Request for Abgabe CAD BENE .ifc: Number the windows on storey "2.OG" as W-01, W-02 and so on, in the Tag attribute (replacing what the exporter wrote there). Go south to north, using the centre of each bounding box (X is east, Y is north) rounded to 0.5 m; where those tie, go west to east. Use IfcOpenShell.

First a look at what the model holds.

```python
import ifcopenshell
import ifcopenshell.util.element
import ifcopenshell.util.placement

model = ifcopenshell.open("Abgabe CAD BENE .ifc")
print(model.schema)
storey = next(s for s in model.by_type("IfcBuildingStorey") if s.Name == "2.OG")
windows = [e for e in ifcopenshell.util.element.get_decomposition(storey) if e.is_a("IfcWindow")]
for e in sorted(windows, key=lambda e: e.id()):
    origin = ifcopenshell.util.placement.get_local_placement(e.ObjectPlacement)[:3, 3]
    print(e.id(), e.Tag, e.Name, origin.round(2) + 0.0, sep=" | ")
```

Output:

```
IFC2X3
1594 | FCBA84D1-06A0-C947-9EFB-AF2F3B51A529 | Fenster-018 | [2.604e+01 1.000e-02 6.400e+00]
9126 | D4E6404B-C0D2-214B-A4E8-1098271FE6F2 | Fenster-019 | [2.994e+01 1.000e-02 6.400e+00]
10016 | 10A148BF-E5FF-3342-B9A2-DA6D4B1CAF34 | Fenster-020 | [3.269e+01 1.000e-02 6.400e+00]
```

```python
import ifcopenshell
import ifcopenshell.geom
import ifcopenshell.util.element
import ifcopenshell.util.shape

model = ifcopenshell.open("Abgabe CAD BENE .ifc")
settings = ifcopenshell.geom.settings()
settings.set("use-world-coords", True)


def centre(element):
    shape = ifcopenshell.geom.create_shape(settings, element)
    return ifcopenshell.util.shape.get_bbox_centroid(shape.geometry)


storey = next(s for s in model.by_type("IfcBuildingStorey") if s.Name == "2.OG")
windows = [e for e in ifcopenshell.util.element.get_decomposition(storey) if e.is_a("IfcWindow")]

# Insertion points can sit at a corner or the storey origin, so sort by the geometry (in metres).
centres = {e: centre(e) for e in windows}
windows.sort(key=lambda e: (round(centres[e][1] / 0.5), centres[e][0]))

for i, e in enumerate(windows, start=1):
    number = f"W-{i:02d}"
    e.Tag = number
    print(e.id(), number)

model.write("Abgabe CAD BENE _edited.ifc")
```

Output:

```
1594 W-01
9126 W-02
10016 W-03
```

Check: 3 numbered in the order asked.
